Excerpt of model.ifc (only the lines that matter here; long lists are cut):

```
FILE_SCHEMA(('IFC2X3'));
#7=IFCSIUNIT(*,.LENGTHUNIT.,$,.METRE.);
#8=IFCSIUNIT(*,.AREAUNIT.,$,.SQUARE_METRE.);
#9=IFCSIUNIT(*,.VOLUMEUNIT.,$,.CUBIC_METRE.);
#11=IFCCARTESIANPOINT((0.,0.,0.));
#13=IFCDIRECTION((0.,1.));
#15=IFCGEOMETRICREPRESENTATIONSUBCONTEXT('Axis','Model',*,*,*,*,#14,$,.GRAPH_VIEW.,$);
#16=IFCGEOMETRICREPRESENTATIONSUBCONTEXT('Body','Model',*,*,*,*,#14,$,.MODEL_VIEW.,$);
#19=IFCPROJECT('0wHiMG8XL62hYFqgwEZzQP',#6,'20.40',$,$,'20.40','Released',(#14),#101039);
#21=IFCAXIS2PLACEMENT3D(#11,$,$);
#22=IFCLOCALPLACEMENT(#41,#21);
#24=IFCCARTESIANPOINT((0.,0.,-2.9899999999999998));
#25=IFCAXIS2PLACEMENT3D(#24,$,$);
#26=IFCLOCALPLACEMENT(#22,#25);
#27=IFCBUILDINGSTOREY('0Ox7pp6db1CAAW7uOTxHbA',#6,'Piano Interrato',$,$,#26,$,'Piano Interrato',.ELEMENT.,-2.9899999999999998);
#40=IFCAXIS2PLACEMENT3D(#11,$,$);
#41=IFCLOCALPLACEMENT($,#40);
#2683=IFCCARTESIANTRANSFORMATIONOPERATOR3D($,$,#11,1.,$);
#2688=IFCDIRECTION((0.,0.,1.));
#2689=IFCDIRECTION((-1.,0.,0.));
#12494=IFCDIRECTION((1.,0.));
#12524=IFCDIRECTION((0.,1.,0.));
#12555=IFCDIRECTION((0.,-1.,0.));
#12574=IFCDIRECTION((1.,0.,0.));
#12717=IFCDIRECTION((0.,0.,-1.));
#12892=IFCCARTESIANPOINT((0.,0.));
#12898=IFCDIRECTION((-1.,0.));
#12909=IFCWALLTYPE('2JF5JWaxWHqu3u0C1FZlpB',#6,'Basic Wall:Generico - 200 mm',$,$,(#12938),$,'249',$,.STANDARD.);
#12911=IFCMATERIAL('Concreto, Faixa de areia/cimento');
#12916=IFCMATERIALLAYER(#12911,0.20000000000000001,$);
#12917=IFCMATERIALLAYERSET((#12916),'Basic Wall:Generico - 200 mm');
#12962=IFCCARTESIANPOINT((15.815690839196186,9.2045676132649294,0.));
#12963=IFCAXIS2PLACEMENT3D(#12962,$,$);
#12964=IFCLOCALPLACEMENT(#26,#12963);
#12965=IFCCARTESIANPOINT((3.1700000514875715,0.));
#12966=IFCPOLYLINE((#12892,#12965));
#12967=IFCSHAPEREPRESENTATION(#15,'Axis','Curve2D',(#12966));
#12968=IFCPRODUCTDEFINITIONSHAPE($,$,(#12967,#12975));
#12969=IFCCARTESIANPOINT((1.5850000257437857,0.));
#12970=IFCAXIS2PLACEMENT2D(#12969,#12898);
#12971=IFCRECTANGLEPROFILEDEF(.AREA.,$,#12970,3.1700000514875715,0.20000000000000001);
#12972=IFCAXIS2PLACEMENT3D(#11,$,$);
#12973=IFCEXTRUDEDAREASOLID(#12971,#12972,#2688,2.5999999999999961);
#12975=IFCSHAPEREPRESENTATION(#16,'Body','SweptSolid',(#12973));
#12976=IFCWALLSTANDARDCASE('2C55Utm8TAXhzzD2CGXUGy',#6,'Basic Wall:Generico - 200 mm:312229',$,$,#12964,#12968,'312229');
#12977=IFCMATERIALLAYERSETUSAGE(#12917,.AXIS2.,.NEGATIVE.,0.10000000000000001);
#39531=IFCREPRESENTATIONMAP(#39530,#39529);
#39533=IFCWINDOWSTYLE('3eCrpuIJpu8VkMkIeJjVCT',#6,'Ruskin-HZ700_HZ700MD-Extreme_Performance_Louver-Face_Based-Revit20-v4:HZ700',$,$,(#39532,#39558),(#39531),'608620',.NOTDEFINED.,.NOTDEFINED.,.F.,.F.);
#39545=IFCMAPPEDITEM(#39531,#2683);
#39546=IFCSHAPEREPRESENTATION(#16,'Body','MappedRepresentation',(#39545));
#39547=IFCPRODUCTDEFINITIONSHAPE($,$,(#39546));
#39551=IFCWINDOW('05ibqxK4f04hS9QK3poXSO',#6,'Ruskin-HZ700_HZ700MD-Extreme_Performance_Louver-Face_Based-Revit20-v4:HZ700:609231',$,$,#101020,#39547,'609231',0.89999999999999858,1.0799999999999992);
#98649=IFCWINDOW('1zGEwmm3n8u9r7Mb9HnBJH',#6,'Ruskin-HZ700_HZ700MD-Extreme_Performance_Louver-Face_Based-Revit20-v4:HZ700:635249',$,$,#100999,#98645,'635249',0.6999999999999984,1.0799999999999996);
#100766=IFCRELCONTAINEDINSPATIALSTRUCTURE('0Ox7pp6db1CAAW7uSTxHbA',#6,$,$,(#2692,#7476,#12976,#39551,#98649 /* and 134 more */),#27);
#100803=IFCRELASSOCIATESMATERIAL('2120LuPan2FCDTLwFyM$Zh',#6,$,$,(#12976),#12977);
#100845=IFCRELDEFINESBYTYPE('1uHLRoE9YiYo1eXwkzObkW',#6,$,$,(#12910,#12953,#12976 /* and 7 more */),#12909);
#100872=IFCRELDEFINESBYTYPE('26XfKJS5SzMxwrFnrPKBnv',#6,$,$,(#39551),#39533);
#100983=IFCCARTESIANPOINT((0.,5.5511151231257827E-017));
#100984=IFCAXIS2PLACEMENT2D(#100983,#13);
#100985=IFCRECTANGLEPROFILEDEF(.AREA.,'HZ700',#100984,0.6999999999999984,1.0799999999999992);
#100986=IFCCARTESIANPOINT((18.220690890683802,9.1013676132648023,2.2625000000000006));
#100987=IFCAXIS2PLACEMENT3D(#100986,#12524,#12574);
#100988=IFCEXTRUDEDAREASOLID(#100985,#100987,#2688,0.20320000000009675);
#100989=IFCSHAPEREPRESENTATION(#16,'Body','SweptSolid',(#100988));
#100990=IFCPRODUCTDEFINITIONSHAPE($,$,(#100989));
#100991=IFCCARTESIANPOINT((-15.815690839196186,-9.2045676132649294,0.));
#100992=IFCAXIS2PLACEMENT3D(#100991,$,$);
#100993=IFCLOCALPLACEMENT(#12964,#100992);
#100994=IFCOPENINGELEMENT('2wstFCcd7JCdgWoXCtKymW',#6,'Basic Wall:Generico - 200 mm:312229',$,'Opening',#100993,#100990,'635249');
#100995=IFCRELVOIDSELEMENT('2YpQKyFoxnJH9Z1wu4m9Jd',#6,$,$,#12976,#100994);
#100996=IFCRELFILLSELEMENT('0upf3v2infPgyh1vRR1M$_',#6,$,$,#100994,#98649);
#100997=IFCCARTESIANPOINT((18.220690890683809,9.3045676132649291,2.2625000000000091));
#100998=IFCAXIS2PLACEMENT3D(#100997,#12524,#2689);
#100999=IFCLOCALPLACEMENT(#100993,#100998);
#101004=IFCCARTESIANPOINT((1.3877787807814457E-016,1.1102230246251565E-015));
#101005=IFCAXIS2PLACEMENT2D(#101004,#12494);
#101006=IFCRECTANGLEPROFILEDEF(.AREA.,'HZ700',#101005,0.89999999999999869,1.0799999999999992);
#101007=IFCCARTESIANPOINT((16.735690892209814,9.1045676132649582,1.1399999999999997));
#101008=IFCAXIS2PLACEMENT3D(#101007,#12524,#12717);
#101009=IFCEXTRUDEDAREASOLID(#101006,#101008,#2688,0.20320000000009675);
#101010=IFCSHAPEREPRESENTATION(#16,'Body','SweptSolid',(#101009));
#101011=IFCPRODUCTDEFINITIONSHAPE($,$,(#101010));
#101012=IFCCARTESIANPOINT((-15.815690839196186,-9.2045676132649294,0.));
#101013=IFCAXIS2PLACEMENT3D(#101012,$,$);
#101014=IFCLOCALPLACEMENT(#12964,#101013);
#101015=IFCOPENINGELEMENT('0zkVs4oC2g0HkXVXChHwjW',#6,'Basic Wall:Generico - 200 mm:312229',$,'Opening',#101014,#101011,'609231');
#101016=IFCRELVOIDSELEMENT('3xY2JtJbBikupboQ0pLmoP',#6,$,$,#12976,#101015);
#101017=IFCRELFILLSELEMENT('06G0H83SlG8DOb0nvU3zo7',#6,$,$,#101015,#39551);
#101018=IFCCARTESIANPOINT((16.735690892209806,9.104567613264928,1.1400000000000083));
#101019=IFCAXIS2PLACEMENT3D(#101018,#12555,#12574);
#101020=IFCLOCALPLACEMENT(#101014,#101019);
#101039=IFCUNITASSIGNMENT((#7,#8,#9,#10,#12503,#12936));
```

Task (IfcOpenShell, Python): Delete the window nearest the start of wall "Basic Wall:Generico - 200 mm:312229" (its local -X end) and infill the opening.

```python
import ifcopenshell
import ifcopenshell.api.feature
import ifcopenshell.api.root
import ifcopenshell.geom
import ifcopenshell.util.shape

model = ifcopenshell.open("model.ifc")
settings = ifcopenshell.geom.settings()


def volume(element):
    """Net volume in cubic metres, openings subtracted."""
    shape = ifcopenshell.geom.create_shape(settings, element)
    return ifcopenshell.util.shape.get_volume(shape.geometry)


window = model.by_guid("05ibqxK4f04hS9QK3poXSO")
opening = window.FillsVoids[0].RelatingOpeningElement
wall = opening.VoidsElements[0].RelatingBuildingElement
before = volume(wall)

ifcopenshell.api.root.remove_product(model, product=window)
ifcopenshell.api.feature.remove_feature(model, feature=opening)

after = volume(wall)

print(f"wall volume {before:.3f} -> {after:.3f} m3")

model.write("model_rev.ifc")
```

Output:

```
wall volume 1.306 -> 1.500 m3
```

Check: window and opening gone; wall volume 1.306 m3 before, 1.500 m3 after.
